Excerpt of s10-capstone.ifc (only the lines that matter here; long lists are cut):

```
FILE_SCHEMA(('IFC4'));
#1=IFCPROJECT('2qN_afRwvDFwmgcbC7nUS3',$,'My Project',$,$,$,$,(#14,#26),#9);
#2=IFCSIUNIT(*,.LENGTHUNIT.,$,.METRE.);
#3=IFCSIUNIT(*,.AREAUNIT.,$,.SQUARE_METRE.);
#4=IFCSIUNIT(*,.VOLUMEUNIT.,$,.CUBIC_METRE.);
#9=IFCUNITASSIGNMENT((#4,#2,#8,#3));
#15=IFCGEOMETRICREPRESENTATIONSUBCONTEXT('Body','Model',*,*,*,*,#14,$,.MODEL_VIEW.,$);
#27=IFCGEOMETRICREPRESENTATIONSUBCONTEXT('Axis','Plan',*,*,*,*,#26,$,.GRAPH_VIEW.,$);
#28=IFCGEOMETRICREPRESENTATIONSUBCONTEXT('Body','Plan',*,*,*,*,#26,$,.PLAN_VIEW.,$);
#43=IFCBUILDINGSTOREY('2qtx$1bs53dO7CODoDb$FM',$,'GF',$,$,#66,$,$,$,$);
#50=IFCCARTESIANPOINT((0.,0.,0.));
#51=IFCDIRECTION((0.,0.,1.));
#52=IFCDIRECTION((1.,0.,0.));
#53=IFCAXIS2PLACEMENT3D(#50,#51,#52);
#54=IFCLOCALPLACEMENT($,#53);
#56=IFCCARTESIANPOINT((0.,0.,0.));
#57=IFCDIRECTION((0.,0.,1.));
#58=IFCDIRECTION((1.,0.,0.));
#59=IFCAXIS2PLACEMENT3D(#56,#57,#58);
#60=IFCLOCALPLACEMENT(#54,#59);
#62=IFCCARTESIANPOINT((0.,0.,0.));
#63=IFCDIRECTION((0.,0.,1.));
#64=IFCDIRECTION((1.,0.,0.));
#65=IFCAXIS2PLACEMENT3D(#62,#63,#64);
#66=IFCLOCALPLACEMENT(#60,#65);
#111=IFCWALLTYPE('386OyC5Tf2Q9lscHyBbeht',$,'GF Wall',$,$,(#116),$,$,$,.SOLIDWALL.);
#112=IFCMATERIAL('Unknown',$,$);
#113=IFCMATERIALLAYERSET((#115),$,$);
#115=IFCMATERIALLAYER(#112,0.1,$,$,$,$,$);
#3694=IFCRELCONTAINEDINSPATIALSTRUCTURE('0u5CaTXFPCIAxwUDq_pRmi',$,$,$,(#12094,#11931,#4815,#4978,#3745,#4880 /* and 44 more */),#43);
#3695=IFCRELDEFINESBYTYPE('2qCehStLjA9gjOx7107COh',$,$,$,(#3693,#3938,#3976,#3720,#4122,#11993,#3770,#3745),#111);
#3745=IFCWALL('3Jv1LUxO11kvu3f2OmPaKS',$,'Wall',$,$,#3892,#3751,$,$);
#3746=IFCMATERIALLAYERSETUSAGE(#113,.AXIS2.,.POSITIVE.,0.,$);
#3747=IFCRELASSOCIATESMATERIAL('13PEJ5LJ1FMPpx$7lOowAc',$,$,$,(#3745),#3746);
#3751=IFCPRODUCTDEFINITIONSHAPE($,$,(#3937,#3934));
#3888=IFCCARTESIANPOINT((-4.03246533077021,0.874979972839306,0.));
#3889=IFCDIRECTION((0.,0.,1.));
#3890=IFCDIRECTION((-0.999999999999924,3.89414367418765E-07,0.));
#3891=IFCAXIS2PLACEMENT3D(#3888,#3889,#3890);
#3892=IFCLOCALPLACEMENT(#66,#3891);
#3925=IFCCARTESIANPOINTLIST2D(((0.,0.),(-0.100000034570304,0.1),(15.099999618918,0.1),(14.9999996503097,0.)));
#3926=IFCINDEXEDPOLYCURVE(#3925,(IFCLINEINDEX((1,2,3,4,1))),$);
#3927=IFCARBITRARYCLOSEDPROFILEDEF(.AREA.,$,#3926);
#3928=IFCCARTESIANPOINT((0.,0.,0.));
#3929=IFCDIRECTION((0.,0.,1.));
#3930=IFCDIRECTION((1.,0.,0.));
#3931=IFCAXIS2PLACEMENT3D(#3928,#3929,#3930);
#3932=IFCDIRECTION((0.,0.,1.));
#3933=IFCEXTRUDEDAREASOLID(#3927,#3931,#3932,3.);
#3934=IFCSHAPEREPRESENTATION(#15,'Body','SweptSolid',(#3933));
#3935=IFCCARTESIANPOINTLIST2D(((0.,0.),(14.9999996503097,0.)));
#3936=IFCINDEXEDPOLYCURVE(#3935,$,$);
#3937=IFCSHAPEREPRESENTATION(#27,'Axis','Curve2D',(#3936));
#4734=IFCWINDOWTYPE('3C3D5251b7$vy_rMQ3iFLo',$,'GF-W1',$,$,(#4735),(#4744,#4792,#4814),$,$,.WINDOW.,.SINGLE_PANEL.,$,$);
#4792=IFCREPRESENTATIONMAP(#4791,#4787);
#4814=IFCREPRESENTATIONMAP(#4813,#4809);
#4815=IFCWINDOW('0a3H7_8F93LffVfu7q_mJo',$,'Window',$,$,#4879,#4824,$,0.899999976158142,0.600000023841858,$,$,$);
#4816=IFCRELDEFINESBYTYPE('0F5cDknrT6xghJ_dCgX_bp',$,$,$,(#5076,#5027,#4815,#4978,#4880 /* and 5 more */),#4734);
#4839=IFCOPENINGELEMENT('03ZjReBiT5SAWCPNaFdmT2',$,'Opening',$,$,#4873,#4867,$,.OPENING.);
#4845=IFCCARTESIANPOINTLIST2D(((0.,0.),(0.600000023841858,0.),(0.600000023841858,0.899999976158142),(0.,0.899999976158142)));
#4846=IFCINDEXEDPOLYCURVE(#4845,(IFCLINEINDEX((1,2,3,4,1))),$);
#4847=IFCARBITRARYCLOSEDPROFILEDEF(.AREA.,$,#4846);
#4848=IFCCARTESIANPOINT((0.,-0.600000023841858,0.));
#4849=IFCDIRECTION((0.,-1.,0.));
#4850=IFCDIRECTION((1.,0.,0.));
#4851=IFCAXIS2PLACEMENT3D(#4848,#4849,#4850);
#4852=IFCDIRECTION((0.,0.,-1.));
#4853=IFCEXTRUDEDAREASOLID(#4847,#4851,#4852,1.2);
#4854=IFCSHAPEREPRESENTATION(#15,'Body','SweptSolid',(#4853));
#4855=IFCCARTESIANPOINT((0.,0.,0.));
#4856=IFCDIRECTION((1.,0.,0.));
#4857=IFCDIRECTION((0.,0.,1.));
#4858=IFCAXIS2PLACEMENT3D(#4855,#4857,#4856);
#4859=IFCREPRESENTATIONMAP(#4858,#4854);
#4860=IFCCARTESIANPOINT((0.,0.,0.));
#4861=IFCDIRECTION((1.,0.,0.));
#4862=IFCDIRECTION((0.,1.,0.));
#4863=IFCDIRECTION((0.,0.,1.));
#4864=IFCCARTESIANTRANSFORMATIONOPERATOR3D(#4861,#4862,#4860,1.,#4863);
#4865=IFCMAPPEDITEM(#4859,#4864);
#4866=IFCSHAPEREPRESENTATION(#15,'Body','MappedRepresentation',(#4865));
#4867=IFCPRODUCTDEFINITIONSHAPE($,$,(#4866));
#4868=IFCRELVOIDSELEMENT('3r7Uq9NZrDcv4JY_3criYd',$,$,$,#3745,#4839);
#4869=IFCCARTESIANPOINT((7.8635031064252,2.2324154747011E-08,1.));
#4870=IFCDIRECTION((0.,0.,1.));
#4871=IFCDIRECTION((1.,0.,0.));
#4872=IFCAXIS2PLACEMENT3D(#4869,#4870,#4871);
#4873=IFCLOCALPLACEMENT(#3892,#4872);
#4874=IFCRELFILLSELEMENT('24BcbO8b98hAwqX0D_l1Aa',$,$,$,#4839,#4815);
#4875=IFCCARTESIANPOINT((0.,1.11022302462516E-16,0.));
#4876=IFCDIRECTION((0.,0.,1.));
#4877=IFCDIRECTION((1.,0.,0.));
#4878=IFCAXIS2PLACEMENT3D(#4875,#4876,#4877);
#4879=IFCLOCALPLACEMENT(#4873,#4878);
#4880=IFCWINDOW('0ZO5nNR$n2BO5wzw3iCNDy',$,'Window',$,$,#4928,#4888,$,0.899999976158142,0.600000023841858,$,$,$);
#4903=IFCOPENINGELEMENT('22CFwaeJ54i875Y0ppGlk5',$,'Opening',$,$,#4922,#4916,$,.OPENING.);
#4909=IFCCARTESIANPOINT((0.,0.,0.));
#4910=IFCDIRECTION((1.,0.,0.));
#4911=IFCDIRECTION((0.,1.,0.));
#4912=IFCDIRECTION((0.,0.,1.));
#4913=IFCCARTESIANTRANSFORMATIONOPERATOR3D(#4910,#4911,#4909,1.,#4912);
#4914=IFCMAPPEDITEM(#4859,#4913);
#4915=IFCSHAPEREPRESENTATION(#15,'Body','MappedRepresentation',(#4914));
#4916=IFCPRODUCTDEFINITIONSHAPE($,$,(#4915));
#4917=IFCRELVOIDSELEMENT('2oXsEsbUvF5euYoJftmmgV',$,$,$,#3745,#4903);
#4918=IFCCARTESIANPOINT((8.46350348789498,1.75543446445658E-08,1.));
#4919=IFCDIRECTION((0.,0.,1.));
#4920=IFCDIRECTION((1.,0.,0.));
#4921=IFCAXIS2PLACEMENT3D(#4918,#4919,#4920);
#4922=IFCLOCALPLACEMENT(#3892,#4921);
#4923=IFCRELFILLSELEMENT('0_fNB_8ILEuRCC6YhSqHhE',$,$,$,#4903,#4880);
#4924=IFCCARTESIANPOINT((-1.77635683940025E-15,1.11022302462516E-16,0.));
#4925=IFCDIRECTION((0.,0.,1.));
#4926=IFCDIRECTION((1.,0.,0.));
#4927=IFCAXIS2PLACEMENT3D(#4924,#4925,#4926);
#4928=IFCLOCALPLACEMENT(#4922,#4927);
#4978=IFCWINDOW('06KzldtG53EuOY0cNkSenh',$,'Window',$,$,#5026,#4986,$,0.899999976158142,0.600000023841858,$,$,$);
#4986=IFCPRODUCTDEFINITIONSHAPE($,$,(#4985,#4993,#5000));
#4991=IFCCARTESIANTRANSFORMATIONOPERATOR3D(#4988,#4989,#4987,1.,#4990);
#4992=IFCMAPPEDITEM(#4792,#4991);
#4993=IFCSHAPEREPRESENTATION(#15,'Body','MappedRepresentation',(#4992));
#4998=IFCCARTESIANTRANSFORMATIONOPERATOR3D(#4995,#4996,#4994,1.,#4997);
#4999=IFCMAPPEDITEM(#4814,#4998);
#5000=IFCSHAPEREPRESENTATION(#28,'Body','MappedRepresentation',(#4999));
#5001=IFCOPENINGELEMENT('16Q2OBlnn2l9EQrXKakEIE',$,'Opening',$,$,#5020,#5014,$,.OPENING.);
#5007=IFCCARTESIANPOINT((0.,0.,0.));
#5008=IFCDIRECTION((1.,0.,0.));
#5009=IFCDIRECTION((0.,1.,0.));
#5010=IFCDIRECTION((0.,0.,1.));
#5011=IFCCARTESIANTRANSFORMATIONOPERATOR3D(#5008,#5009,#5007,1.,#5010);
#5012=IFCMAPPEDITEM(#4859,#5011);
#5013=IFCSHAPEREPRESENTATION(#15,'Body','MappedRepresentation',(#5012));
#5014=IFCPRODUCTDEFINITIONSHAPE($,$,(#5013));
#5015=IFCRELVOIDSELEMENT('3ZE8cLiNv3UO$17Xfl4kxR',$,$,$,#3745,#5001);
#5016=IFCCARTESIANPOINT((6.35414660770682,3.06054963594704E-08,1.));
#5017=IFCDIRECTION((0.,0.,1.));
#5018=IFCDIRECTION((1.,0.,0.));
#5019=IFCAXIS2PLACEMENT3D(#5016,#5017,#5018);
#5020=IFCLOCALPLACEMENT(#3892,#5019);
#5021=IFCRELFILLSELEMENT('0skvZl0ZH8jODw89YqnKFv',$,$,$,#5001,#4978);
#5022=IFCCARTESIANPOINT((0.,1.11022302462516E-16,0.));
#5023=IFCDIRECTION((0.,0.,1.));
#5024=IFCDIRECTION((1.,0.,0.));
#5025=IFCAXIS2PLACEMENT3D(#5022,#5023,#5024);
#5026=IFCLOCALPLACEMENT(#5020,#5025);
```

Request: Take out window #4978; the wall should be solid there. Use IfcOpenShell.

```python
import ifcopenshell
import ifcopenshell.api.feature
import ifcopenshell.api.root
import ifcopenshell.geom
import ifcopenshell.util.shape

model = ifcopenshell.open("s10-capstone.ifc")
settings = ifcopenshell.geom.settings()


def volume(element):
    """Net volume in cubic metres, openings subtracted."""
    shape = ifcopenshell.geom.create_shape(settings, element)
    return ifcopenshell.util.shape.get_volume(shape.geometry)


window = model.by_guid("06KzldtG53EuOY0cNkSenh")
opening = window.FillsVoids[0].RelatingOpeningElement
wall = opening.VoidsElements[0].RelatingBuildingElement
before = volume(wall)

ifcopenshell.api.root.remove_product(model, product=window)
ifcopenshell.api.feature.remove_feature(model, feature=opening)

after = volume(wall)

print(f"wall volume {before:.3f} -> {after:.3f} m3")

model.write("s10-capstone_edited.ifc")
```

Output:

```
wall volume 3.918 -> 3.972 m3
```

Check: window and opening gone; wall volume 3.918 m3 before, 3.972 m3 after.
